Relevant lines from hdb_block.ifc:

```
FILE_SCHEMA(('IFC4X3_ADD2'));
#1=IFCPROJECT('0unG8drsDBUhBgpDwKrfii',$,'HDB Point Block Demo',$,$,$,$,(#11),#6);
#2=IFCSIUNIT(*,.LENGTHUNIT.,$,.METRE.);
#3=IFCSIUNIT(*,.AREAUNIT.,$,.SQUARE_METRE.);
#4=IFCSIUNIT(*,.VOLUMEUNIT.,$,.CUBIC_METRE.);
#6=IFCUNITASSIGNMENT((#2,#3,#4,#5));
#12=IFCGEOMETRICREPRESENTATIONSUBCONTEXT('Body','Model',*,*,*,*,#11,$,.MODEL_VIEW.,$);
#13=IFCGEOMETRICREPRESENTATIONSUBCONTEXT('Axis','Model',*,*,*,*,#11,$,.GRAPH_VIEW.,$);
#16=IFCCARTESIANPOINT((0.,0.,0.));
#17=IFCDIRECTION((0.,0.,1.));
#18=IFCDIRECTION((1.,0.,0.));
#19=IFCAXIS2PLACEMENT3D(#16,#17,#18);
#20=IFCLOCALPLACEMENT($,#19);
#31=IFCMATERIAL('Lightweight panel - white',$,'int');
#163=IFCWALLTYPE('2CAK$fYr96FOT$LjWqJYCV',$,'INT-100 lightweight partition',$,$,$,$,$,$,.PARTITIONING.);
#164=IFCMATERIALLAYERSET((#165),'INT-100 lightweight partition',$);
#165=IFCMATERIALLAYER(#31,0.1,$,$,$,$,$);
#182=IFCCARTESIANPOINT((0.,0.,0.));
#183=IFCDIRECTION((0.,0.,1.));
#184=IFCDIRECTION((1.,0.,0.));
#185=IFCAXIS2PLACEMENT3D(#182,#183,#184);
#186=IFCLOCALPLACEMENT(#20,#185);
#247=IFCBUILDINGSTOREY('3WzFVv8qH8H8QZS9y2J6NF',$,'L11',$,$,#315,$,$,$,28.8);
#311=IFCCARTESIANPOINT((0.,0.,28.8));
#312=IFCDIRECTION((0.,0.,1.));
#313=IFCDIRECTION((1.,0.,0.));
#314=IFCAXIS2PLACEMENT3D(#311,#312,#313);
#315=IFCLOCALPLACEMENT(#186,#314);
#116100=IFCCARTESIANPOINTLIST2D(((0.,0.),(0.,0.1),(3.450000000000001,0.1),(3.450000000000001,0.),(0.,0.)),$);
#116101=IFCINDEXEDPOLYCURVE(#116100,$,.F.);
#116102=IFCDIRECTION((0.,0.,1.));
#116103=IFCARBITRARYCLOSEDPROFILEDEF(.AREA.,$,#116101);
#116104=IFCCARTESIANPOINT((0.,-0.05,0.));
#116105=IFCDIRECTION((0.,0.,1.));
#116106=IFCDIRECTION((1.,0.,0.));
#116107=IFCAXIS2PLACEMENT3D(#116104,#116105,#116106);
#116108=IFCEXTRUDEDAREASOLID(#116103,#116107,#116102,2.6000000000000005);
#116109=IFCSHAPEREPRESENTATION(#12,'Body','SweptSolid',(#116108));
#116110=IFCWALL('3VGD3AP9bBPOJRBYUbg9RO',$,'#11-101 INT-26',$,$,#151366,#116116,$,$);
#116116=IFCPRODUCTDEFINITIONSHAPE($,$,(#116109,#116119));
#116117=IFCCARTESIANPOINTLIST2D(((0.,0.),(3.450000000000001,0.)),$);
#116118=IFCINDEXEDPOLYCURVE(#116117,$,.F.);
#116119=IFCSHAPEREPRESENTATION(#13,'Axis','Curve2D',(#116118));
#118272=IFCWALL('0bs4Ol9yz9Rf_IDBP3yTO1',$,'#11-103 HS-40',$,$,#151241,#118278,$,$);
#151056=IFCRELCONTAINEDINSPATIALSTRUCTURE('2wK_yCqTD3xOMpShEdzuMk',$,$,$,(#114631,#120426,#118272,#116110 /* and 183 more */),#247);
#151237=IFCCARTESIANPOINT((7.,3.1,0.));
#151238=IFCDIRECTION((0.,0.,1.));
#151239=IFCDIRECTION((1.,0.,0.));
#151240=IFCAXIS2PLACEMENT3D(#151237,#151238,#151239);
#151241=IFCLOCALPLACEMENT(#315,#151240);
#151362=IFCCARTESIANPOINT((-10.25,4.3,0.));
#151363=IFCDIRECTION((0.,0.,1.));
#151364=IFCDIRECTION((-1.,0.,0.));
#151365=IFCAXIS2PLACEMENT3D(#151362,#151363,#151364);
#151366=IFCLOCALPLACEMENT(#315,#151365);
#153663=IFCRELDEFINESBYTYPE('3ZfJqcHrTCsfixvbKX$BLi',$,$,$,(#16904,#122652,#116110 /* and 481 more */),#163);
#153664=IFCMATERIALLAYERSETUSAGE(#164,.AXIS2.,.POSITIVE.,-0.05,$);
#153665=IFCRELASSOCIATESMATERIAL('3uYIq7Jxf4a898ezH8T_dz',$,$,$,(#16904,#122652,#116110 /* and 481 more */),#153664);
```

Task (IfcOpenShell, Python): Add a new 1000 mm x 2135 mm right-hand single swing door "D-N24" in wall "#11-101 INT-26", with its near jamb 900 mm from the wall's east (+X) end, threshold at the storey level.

```python
import numpy as np
import ifcopenshell
import ifcopenshell.api.feature
import ifcopenshell.api.geometry
import ifcopenshell.api.root
import ifcopenshell.api.spatial
import ifcopenshell.geom
import ifcopenshell.util.element
import ifcopenshell.util.placement
import ifcopenshell.util.representation
import ifcopenshell.util.shape
import ifcopenshell.util.unit

model = ifcopenshell.open("hdb_block.ifc")
unit_scale = ifcopenshell.util.unit.calculate_unit_scale(model)
settings = ifcopenshell.geom.settings()


def volume(element):
    """Net volume in cubic metres, openings subtracted."""
    shape = ifcopenshell.geom.create_shape(settings, element)
    return ifcopenshell.util.shape.get_volume(shape.geometry)


wall = model.by_guid("3VGD3AP9bBPOJRBYUbg9RO")
storey = ifcopenshell.util.element.get_container(wall, ifc_class="IfcBuildingStorey")
context = ifcopenshell.util.representation.get_context(model, "Model", "Body", "MODEL_VIEW")
before = volume(wall)

width, height, from_end, sill = 1, 2.135, 0.9, 0.0  # metres

# The wall runs along its own X axis, and the end named is its -X end.
wall_shape = ifcopenshell.geom.create_shape(settings, wall)
x, y, z = ifcopenshell.util.shape.get_vertices(wall_shape.geometry).T
start = x.min() + from_end
face, thickness = float(y.min()), float(y.max() - y.min())
wall_matrix = ifcopenshell.util.placement.get_local_placement(wall.ObjectPlacement)
level = ifcopenshell.util.placement.get_local_placement(storey.ObjectPlacement)[2, 3]


def in_wall(x, y):
    """Placement at x, y metres in the wall's axes, at sill height."""
    matrix = wall_matrix.copy()
    matrix[:, 3] = wall_matrix @ np.array([x / unit_scale, y / unit_scale, 0.0, 1.0])
    matrix[2, 3] = level + sill / unit_scale
    return matrix


# Opening: a box that overshoots both wall faces by 50 mm.
opening = ifcopenshell.api.root.create_entity(model, ifc_class="IfcOpeningElement", predefined_type="OPENING")
box = ifcopenshell.api.geometry.add_wall_representation(
    model, context=context, length=width, height=height, thickness=thickness + 0.1
)
ifcopenshell.api.geometry.assign_representation(model, product=opening, representation=box)
ifcopenshell.api.geometry.edit_object_placement(model, product=opening, matrix=in_wall(start, face - 0.05), is_si=False)
ifcopenshell.api.feature.add_feature(model, feature=opening, element=wall)

door = ifcopenshell.api.root.create_entity(model, ifc_class="IfcDoor", name="D-N24", predefined_type="DOOR")
door.OverallWidth, door.OverallHeight = width / unit_scale, height / unit_scale
door.OperationType = "SINGLE_SWING_RIGHT"
body = ifcopenshell.api.geometry.add_door_representation(
    model,
    context=context,
    overall_width=door.OverallWidth,
    overall_height=door.OverallHeight,
    operation_type="SINGLE_SWING_RIGHT",
    lining_properties={"LiningDepth": thickness / unit_scale, "ThresholdDepth": thickness / unit_scale},
)
ifcopenshell.api.geometry.assign_representation(model, product=door, representation=body)
ifcopenshell.api.spatial.assign_container(model, products=[door], relating_structure=storey)
ifcopenshell.api.feature.add_filling(model, opening=opening, element=door)

# The lining spans the wall, so the door starts at the wall face.
ifcopenshell.api.geometry.edit_object_placement(model, product=door, matrix=in_wall(start, face), is_si=False)

after = volume(wall)

print(f"wall volume {before:.3f} -> {after:.3f} m3")

model.write("hdb_block_edited.ifc")
```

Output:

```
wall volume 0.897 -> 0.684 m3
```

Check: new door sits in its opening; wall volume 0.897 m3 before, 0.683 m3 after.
